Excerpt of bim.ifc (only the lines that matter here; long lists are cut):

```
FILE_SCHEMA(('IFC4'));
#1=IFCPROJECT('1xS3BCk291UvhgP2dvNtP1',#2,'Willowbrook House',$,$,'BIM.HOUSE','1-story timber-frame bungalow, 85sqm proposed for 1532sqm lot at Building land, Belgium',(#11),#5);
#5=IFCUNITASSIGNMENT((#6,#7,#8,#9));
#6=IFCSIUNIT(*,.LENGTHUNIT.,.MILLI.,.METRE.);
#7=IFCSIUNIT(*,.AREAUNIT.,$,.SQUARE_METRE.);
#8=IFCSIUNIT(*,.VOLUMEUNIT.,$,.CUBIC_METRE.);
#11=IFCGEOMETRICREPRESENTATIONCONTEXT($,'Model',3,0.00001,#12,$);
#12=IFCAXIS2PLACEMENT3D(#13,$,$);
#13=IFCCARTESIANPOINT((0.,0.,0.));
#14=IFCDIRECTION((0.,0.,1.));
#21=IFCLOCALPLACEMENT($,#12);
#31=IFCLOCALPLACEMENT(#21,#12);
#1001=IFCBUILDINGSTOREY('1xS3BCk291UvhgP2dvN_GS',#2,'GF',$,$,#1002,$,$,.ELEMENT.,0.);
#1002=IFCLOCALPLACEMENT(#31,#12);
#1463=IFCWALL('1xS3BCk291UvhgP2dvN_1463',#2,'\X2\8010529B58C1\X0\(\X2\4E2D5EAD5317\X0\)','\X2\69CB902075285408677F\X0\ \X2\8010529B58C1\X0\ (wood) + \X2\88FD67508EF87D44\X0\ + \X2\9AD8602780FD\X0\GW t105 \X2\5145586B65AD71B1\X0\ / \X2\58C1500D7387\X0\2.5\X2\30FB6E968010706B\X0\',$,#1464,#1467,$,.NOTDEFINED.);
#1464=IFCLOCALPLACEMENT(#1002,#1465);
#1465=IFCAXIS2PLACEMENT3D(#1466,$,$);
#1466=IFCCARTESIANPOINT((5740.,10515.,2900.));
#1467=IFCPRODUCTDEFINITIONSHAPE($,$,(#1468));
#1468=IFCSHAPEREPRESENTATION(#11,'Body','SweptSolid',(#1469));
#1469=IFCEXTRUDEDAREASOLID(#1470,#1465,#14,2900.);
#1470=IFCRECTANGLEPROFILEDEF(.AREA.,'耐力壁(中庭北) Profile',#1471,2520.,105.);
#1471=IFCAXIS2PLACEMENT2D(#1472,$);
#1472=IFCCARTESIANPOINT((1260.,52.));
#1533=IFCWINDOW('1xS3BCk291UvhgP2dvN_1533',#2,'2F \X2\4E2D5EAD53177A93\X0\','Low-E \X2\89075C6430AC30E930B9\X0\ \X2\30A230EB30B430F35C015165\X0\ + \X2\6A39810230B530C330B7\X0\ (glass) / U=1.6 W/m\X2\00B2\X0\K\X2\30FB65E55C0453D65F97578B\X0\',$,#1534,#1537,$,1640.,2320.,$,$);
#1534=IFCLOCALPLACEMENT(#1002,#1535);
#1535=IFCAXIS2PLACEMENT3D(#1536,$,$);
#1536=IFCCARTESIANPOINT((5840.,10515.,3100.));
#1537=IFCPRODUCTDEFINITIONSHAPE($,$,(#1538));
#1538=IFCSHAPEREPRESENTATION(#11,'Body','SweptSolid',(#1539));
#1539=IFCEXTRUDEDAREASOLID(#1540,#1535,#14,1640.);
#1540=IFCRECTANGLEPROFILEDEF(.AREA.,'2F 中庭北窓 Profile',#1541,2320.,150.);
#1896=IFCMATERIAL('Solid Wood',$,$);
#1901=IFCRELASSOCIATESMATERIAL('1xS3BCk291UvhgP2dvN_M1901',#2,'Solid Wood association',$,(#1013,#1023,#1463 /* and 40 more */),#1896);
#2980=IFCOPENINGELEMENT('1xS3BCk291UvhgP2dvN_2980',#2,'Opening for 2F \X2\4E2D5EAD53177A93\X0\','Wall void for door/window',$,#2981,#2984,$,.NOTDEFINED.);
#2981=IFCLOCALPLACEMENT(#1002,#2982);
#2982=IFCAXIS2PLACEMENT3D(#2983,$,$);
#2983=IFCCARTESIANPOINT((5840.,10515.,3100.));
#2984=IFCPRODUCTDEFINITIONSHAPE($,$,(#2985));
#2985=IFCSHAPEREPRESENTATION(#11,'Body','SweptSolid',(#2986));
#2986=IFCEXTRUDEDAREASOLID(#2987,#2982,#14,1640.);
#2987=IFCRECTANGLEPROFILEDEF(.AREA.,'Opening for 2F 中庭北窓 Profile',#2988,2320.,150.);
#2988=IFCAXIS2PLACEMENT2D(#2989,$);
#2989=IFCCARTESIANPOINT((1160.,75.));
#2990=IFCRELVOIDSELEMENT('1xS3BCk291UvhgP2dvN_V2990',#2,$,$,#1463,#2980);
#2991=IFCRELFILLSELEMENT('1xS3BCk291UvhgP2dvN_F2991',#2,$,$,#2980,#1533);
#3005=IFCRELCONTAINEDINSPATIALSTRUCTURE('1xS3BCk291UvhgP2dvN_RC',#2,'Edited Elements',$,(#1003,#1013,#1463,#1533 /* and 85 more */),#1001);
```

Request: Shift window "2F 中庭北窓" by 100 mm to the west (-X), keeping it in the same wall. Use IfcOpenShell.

```python
import ifcopenshell
import ifcopenshell.api.geometry
import ifcopenshell.util.placement
import ifcopenshell.util.unit

model = ifcopenshell.open("bim.ifc")
unit_scale = ifcopenshell.util.unit.calculate_unit_scale(model)

window = model.by_guid("1xS3BCk291UvhgP2dvN_1533")
opening = window.FillsVoids[0].RelatingOpeningElement
wall = opening.VoidsElements[0].RelatingBuildingElement

wall_matrix = ifcopenshell.util.placement.get_local_placement(wall.ObjectPlacement)
shift = wall_matrix[:3, 0] * -0.1 / unit_scale
before = ifcopenshell.util.placement.get_local_placement(window.ObjectPlacement)[:3, 3].copy()

# The window is not placed relative to its opening, so move both.
for product in (opening, window):
    matrix = ifcopenshell.util.placement.get_local_placement(product.ObjectPlacement)
    matrix[:3, 3] += shift
    ifcopenshell.api.geometry.edit_object_placement(model, product=product, matrix=matrix, is_si=False)

after = ifcopenshell.util.placement.get_local_placement(window.ObjectPlacement)[:3, 3]
print("window moved by", (after - before).round(3) + 0.0)

model.write("bim-out.ifc")
```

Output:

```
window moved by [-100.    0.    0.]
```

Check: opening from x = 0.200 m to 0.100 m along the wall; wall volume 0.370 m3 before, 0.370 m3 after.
